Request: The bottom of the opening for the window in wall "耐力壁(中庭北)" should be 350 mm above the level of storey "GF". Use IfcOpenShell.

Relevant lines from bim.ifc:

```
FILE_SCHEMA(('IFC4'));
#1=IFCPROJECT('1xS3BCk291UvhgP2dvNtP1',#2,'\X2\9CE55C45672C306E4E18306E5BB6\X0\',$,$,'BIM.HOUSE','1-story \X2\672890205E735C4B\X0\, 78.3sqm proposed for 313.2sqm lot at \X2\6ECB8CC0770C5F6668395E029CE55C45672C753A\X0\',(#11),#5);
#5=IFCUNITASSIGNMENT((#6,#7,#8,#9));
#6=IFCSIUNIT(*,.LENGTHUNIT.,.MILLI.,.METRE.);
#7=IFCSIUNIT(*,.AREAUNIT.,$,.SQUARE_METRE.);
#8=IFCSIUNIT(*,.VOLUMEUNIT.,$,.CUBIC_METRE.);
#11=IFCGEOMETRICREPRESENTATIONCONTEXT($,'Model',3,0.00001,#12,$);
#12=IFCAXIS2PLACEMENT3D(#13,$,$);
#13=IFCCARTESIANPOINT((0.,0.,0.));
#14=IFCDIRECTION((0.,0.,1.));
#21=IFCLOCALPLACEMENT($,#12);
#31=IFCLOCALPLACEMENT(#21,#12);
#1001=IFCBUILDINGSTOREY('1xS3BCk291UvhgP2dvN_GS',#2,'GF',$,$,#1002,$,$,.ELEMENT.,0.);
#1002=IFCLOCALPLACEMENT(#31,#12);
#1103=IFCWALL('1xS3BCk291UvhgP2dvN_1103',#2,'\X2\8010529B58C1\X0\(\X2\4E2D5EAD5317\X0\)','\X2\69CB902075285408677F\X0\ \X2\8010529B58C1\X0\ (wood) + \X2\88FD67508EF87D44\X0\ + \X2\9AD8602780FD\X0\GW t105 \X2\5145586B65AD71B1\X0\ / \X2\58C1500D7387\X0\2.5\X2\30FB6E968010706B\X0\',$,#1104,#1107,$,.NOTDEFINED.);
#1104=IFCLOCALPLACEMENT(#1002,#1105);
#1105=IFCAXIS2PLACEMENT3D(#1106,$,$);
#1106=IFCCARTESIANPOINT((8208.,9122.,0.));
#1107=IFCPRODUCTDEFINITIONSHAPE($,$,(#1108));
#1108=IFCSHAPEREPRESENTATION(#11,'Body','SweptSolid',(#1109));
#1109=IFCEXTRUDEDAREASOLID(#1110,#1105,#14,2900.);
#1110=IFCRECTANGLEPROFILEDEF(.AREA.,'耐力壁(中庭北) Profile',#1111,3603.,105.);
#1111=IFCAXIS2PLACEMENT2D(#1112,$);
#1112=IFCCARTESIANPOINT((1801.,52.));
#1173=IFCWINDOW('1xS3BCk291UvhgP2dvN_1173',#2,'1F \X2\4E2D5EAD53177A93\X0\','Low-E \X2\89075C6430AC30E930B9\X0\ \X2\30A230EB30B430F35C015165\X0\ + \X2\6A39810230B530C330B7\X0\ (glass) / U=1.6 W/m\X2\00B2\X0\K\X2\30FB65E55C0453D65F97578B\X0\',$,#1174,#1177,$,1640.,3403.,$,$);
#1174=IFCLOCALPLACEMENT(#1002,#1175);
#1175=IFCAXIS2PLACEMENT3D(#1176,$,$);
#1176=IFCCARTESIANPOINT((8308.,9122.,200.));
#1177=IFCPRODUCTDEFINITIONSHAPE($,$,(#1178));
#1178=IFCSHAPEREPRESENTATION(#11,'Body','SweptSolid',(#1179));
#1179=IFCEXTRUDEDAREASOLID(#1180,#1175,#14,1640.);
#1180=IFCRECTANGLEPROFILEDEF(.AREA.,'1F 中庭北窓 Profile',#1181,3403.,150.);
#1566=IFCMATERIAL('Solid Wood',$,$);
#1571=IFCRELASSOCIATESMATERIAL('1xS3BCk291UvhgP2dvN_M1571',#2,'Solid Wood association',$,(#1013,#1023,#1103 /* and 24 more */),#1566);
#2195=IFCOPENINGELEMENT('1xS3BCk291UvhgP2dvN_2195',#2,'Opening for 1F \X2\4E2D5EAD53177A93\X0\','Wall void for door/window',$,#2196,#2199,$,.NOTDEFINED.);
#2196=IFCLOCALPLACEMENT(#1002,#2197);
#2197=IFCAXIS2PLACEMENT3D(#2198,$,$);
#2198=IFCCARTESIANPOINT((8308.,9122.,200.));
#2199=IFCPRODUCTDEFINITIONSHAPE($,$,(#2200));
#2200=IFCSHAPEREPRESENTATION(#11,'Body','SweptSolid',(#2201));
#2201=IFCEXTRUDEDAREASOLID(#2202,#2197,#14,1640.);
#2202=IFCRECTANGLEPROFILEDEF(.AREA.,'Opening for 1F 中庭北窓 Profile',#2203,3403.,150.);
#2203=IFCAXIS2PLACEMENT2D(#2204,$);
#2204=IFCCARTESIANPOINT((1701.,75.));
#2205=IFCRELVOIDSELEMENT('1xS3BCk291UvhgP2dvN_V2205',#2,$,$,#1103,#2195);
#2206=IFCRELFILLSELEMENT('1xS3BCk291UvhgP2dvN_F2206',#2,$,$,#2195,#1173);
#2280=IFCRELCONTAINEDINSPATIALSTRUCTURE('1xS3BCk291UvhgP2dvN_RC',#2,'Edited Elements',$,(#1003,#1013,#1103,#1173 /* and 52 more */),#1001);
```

```python
import numpy as np
import ifcopenshell
import ifcopenshell.api.geometry
import ifcopenshell.geom
import ifcopenshell.util.element
import ifcopenshell.util.placement
import ifcopenshell.util.shape
import ifcopenshell.util.unit

model = ifcopenshell.open("bim.ifc")
unit_scale = ifcopenshell.util.unit.calculate_unit_scale(model)

window = model.by_id(1173)
opening = window.FillsVoids[0].RelatingOpeningElement
storey = ifcopenshell.util.element.get_container(window, ifc_class="IfcBuildingStorey")
level = ifcopenshell.util.placement.get_local_placement(storey.ObjectPlacement)[2, 3]

# The opening's origin need not be at the sill, so measure its lowest point.
shape = ifcopenshell.geom.create_shape(ifcopenshell.geom.settings(), opening)
bottom = ifcopenshell.util.shape.get_shape_bottom_elevation(shape, shape.geometry) / unit_scale
dz = level + 350.0 - bottom

shift = np.array([0.0, 0.0, dz])
# The window is not placed relative to its opening, so move both.
for product in (opening, window):
    matrix = ifcopenshell.util.placement.get_local_placement(product.ObjectPlacement)
    matrix[:3, 3] += shift
    ifcopenshell.api.geometry.edit_object_placement(model, product=product, matrix=matrix, is_si=False)

print(f"moved by {dz * unit_scale:+.3f} m")

model.write("bim_edited.ifc")
```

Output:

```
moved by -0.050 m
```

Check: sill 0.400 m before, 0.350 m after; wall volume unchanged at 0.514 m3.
